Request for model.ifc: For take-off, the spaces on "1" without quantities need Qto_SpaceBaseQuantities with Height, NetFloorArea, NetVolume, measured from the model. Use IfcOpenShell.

First a look at what the model holds.

```python
import ifcopenshell
import ifcopenshell.util.element
import ifcopenshell.util.unit

model = ifcopenshell.open("model.ifc")
print(model.schema)
for unit_type in ("LENGTHUNIT", "AREAUNIT", "VOLUMEUNIT"):
    print(unit_type, ifcopenshell.util.unit.calculate_unit_scale(model, unit_type))
storey = next(s for s in model.by_type("IfcBuildingStorey") if s.Name == "1")
spaces = [e for e in ifcopenshell.util.element.get_decomposition(storey) if e.is_a("IfcSpace")]
for e in sorted(spaces, key=lambda e: e.id()):
    print(e.id(), e.is_a(), e.Name, list(ifcopenshell.util.element.get_psets(e, qtos_only=True)), sep=" | ")
```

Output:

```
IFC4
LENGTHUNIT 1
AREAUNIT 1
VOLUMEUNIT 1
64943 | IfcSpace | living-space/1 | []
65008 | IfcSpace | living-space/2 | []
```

```python
import ifcopenshell
import ifcopenshell.api.pset
import ifcopenshell.geom
import ifcopenshell.util.element
import ifcopenshell.util.shape
import ifcopenshell.util.unit

model = ifcopenshell.open("model.ifc")
unit_scale = ifcopenshell.util.unit.calculate_unit_scale(model)
area_scale = ifcopenshell.util.unit.calculate_unit_scale(model, "AREAUNIT")
volume_scale = ifcopenshell.util.unit.calculate_unit_scale(model, "VOLUMEUNIT")
settings = ifcopenshell.geom.settings()

storey = next(s for s in model.by_type("IfcBuildingStorey") if s.Name == "1")
spaces = [e for e in ifcopenshell.util.element.get_decomposition(storey) if e.is_a("IfcSpace")]

for e in sorted(spaces, key=lambda e: e.id()):
    if ifcopenshell.util.element.get_psets(e, qtos_only=True, should_inherit=False):
        continue
    # Geometry comes back in metres, in the element's own axes.
    shape = ifcopenshell.geom.create_shape(settings, e)
    values = {
        "Height": ifcopenshell.util.shape.get_z(shape.geometry) / unit_scale,
        "NetFloorArea": ifcopenshell.util.shape.get_footprint_area(shape.geometry) / area_scale,
        "NetVolume": ifcopenshell.util.shape.get_volume(shape.geometry) / volume_scale,
    }
    qto = ifcopenshell.api.pset.add_qto(model, product=e, name="Qto_SpaceBaseQuantities")
    ifcopenshell.api.pset.edit_qto(model, qto=qto, properties=values)
    print(e.id(), {k: round(v, 3) for k, v in values.items()})

model.write("model-out.ifc")
```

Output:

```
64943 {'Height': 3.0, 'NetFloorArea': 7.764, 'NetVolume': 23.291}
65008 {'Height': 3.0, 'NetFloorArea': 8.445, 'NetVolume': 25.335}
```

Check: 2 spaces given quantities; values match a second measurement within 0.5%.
